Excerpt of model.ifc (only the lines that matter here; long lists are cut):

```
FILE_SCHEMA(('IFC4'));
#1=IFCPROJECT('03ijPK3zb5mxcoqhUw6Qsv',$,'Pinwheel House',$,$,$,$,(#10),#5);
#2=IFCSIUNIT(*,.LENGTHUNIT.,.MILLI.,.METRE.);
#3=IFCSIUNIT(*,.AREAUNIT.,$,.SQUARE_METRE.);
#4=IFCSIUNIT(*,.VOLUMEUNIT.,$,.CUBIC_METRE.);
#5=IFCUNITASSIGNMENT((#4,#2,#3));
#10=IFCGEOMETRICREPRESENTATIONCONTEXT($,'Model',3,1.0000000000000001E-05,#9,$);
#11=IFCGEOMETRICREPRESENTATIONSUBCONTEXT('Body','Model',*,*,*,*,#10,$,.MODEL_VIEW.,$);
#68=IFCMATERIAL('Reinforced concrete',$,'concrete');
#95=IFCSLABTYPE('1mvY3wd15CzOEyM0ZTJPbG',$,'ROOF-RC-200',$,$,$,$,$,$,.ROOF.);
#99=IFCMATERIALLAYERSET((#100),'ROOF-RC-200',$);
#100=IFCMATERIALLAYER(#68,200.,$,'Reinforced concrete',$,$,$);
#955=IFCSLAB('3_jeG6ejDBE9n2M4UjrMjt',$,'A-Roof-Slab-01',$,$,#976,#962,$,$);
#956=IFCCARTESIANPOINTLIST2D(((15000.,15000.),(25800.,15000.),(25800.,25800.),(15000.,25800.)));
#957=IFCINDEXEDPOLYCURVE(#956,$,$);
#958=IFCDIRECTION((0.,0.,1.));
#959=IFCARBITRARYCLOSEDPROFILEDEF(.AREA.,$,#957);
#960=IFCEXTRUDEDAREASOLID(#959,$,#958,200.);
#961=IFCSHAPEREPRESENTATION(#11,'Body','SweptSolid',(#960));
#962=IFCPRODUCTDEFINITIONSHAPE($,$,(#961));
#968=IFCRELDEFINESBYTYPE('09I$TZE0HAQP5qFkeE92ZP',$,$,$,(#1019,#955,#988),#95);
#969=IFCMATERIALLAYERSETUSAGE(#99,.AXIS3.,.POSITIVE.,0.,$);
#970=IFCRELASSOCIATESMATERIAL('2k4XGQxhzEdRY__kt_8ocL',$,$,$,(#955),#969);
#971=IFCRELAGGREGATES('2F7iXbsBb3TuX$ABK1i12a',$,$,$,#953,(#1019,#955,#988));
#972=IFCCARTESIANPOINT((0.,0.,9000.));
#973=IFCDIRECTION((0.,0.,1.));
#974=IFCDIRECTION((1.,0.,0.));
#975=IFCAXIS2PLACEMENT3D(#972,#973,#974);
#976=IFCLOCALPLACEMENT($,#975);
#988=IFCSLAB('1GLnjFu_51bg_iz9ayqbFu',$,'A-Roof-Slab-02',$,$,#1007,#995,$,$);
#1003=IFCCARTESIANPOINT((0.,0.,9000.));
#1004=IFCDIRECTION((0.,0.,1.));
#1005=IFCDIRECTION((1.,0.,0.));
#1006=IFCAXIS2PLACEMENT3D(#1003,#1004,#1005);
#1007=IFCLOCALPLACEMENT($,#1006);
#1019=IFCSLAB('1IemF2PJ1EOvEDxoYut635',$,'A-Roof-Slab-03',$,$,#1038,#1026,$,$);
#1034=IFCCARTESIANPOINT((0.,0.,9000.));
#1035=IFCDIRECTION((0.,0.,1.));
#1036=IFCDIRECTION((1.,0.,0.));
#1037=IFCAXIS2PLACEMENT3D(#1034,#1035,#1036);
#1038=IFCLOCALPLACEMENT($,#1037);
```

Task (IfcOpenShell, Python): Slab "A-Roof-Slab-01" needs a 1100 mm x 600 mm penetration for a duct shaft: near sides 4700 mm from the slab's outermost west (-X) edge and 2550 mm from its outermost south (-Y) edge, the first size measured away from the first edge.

```python
import numpy as np
import ifcopenshell
import ifcopenshell.api.feature
import ifcopenshell.api.geometry
import ifcopenshell.api.root
import ifcopenshell.geom
import ifcopenshell.util.placement
import ifcopenshell.util.representation
import ifcopenshell.util.shape
import ifcopenshell.util.unit

model = ifcopenshell.open("model.ifc")
unit_scale = ifcopenshell.util.unit.calculate_unit_scale(model)
settings = ifcopenshell.geom.settings()


def volume(element):
    """Net volume in cubic metres, openings subtracted."""
    shape = ifcopenshell.geom.create_shape(settings, element)
    return ifcopenshell.util.shape.get_volume(shape.geometry)


slab = model.by_id(955)
before = volume(slab)

# Extent in the slab's own axes, in metres. The edges named are its -X and -Y sides.
slab_shape = ifcopenshell.geom.create_shape(settings, slab)
vertices = ifcopenshell.util.shape.get_vertices(slab_shape.geometry)
x_min, y_min, bottom = vertices.min(axis=0)
top = vertices[:, 2].max()

opening = ifcopenshell.api.root.create_entity(model, ifc_class="IfcOpeningElement", name="Duct shaft opening", predefined_type="OPENING")
context = ifcopenshell.util.representation.get_context(model, "Model", "Body", "MODEL_VIEW")
width, depth = 1.1, 0.6
outline = [(0.0, 0.0), (width, 0.0), (width, depth), (0.0, depth), (0.0, 0.0)]
# Overshoot both faces by 50 mm so the cut is clean.
shape = ifcopenshell.api.geometry.add_slab_representation(
    model, context=context, depth=top - bottom + 0.1, polyline=outline
)
ifcopenshell.api.geometry.assign_representation(model, product=opening, representation=shape)

matrix = ifcopenshell.util.placement.get_local_placement(slab.ObjectPlacement)
matrix[:, 3] = matrix @ np.append(np.array([x_min + 4.7, y_min + 2.55, bottom - 0.05]) / unit_scale, 1.0)
ifcopenshell.api.geometry.edit_object_placement(model, product=opening, matrix=matrix, is_si=False)
ifcopenshell.api.feature.add_feature(model, feature=opening, element=slab)

after = volume(slab)

print(f"slab volume {before:.3f} -> {after:.3f} m3")

model.write("model_updated.ifc")
```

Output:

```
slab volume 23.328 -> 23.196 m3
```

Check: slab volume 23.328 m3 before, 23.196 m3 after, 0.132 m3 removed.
